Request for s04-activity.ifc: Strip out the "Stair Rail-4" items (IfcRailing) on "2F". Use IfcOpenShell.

First a look at what the model holds.

```python
import ifcopenshell
import ifcopenshell.util.element

model = ifcopenshell.open("s04-activity.ifc")
print(model.schema)
storey = next(s for s in model.by_type("IfcBuildingStorey") if s.Name == "2F")
railings = [e for e in ifcopenshell.util.element.get_decomposition(storey) if e.is_a("IfcRailing")]
seen = {}
for e in railings:
    element_type = ifcopenshell.util.element.get_type(e)
    name = element_type.Name if element_type not in (None, e) else None
    seen[name] = seen.get(name, 0) + 1
for name, count in sorted(seen.items(), key=str):
    print(count, "x", name)
```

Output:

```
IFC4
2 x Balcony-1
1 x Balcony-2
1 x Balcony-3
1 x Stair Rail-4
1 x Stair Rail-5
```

```python
import ifcopenshell
import ifcopenshell.api.root
import ifcopenshell.util.element

model = ifcopenshell.open("s04-activity.ifc")

storey = next(s for s in model.by_type("IfcBuildingStorey") if s.Name == "2F")
railings = [e for e in ifcopenshell.util.element.get_decomposition(storey) if e.is_a("IfcRailing")]
targets = [e for e in railings if (t := ifcopenshell.util.element.get_type(e)) not in (None, e) and t.Name == "Stair Rail-4"]

for e in targets:
    ifcopenshell.api.root.remove_product(model, product=e)
print(len(targets), "removed")

model.write("s04-activity_v2.ifc")
```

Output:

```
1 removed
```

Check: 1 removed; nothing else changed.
